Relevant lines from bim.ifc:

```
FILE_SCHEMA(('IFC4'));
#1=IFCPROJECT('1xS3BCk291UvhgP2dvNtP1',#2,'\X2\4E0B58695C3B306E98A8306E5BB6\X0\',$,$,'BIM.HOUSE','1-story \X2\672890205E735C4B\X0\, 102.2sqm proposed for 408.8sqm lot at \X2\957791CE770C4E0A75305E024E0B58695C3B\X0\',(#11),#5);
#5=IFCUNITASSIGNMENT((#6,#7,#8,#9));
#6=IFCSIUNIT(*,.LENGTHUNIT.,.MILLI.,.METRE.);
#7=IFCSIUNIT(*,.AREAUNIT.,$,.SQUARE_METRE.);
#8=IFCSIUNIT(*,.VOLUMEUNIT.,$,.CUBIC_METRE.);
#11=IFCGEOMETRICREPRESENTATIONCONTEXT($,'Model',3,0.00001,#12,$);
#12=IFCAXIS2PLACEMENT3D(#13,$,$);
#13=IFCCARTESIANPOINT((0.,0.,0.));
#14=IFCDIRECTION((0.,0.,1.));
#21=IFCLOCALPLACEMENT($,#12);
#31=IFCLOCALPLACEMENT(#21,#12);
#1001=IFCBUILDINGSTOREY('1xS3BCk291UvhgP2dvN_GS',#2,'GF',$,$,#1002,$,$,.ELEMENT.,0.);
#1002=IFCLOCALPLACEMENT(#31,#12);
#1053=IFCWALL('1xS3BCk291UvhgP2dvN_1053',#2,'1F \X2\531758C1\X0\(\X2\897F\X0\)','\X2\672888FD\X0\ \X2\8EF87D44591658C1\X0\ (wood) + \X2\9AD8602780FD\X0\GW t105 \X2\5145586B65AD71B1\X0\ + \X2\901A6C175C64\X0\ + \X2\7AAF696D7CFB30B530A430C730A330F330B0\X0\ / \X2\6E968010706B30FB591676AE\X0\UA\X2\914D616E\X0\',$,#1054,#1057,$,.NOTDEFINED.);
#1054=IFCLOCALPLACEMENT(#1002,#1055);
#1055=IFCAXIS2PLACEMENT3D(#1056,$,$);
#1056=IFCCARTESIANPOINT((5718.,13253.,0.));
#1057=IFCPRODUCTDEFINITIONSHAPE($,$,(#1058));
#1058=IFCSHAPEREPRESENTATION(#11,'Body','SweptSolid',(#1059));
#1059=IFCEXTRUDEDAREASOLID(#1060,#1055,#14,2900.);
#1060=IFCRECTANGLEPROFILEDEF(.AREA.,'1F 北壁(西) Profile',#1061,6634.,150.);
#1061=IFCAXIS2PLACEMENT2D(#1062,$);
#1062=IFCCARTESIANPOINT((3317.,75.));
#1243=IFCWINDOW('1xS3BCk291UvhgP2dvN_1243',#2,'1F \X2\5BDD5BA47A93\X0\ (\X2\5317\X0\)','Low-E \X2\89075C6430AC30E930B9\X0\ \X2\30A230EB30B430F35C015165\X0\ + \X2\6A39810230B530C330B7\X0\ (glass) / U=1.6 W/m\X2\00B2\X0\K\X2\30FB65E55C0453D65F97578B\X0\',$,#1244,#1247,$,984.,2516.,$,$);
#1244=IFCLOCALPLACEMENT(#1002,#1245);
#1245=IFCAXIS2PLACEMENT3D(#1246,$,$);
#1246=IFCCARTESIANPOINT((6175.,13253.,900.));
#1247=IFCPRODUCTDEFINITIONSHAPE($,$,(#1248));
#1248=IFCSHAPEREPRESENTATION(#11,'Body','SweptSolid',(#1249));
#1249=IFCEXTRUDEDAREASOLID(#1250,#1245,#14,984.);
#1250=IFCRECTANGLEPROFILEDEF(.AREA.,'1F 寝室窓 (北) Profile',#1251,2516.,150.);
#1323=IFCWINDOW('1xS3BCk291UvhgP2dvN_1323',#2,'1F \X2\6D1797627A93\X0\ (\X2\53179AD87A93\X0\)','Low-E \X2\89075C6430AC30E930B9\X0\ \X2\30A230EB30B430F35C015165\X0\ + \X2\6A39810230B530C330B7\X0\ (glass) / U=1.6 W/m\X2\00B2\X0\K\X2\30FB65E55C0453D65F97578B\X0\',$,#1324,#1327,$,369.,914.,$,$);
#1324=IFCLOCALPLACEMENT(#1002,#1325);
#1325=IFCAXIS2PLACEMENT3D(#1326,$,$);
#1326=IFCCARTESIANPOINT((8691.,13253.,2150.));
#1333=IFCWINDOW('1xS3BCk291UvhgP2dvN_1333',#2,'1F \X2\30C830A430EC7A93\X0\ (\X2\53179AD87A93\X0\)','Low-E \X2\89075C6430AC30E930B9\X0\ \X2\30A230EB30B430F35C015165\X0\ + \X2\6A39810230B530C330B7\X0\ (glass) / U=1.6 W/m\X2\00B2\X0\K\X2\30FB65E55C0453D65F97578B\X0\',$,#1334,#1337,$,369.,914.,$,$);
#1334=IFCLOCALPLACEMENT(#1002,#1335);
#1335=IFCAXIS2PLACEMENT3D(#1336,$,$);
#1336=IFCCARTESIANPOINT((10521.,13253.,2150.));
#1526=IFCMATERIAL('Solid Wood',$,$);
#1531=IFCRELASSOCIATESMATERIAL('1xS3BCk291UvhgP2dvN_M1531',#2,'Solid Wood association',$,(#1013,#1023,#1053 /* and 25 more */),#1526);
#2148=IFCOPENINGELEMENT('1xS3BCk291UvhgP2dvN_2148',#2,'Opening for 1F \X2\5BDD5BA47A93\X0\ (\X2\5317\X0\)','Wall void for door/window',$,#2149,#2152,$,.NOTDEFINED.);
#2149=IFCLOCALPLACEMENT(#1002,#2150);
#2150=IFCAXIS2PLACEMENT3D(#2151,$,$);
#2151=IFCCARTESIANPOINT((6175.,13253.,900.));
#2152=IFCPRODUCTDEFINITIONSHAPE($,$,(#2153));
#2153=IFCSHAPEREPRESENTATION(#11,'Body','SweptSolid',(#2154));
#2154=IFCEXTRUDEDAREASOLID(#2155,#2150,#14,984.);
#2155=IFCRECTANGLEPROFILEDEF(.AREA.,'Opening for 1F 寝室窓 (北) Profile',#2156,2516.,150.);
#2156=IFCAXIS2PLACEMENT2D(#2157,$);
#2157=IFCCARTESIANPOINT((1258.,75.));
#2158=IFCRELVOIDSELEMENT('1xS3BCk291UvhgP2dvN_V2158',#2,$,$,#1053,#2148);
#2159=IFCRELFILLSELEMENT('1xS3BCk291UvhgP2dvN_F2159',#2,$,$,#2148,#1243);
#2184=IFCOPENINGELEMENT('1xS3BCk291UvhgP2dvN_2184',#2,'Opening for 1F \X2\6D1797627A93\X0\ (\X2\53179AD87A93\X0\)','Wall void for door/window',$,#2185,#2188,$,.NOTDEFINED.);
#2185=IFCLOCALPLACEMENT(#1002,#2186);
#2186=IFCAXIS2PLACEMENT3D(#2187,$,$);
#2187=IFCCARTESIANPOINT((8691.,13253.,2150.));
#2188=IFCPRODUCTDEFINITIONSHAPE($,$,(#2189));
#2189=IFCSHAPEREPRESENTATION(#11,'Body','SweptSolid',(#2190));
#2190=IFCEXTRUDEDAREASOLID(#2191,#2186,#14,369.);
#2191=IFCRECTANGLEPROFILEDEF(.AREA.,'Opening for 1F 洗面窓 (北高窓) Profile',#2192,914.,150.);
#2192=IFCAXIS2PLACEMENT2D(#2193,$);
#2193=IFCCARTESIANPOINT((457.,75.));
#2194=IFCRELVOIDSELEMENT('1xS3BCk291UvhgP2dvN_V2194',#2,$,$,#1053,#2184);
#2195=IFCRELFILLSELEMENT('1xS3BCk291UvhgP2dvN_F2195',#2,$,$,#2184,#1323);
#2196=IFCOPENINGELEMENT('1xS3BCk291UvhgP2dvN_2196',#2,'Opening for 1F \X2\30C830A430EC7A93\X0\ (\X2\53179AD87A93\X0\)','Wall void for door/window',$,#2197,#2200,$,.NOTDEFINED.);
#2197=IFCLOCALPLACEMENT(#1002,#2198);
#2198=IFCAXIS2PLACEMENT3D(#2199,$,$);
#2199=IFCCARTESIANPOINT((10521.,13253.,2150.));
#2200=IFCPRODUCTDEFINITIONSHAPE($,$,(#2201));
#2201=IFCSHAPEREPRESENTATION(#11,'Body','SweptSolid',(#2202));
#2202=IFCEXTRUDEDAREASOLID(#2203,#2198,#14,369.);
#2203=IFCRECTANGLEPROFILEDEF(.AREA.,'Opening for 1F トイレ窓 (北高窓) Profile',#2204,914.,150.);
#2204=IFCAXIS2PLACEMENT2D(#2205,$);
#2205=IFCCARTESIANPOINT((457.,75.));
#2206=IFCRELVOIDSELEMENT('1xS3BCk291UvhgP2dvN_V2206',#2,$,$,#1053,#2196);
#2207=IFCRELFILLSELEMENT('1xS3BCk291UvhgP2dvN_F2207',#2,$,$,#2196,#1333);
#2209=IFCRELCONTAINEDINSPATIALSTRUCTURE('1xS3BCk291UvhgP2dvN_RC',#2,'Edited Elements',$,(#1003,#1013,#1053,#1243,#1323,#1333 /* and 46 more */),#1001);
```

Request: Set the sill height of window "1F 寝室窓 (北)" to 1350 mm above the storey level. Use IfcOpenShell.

```python
import numpy as np
import ifcopenshell
import ifcopenshell.api.geometry
import ifcopenshell.geom
import ifcopenshell.util.element
import ifcopenshell.util.placement
import ifcopenshell.util.shape
import ifcopenshell.util.unit

model = ifcopenshell.open("bim.ifc")
unit_scale = ifcopenshell.util.unit.calculate_unit_scale(model)

window = model.by_guid("1xS3BCk291UvhgP2dvN_1243")
opening = window.FillsVoids[0].RelatingOpeningElement
storey = ifcopenshell.util.element.get_container(window, ifc_class="IfcBuildingStorey")
level = ifcopenshell.util.placement.get_local_placement(storey.ObjectPlacement)[2, 3]

# The opening's origin need not be at the sill, so measure its lowest point.
shape = ifcopenshell.geom.create_shape(ifcopenshell.geom.settings(), opening)
bottom = ifcopenshell.util.shape.get_shape_bottom_elevation(shape, shape.geometry) / unit_scale
dz = level + 1.35 / unit_scale - bottom

shift = np.array([0.0, 0.0, dz])
# The window is not placed relative to its opening, so move both.
for product in (opening, window):
    matrix = ifcopenshell.util.placement.get_local_placement(product.ObjectPlacement)
    matrix[:3, 3] += shift
    ifcopenshell.api.geometry.edit_object_placement(model, product=product, matrix=matrix, is_si=False)

print(f"moved by {dz * unit_scale:+.3f} m")

model.write("bim_rev.ifc")
```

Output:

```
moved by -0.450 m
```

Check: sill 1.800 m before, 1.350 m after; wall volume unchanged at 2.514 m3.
